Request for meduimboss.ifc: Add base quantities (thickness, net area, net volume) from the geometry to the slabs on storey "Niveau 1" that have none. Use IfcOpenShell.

First a look at what the model holds.

```python
import ifcopenshell
import ifcopenshell.util.element
import ifcopenshell.util.unit

model = ifcopenshell.open("meduimboss.ifc")
print(model.schema)
for unit_type in ("LENGTHUNIT", "AREAUNIT", "VOLUMEUNIT"):
    print(unit_type, ifcopenshell.util.unit.calculate_unit_scale(model, unit_type))
storey = next(s for s in model.by_type("IfcBuildingStorey") if s.Name == "Niveau 1")
slabs = [e for e in ifcopenshell.util.element.get_decomposition(storey) if e.is_a("IfcSlab")]
for e in sorted(slabs, key=lambda e: e.id()):
    print(e.id(), e.is_a(), e.Name, list(ifcopenshell.util.element.get_psets(e, qtos_only=True)), sep=" | ")
```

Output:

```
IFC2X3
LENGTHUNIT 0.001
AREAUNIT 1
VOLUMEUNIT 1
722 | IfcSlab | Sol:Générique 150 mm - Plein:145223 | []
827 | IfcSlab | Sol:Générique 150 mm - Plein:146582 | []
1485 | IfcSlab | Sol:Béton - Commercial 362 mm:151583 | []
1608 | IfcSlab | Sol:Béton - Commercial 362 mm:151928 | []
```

```python
import ifcopenshell
import ifcopenshell.api.pset
import ifcopenshell.geom
import ifcopenshell.util.element
import ifcopenshell.util.shape
import ifcopenshell.util.unit

model = ifcopenshell.open("meduimboss.ifc")
unit_scale = ifcopenshell.util.unit.calculate_unit_scale(model)
area_scale = ifcopenshell.util.unit.calculate_unit_scale(model, "AREAUNIT")
volume_scale = ifcopenshell.util.unit.calculate_unit_scale(model, "VOLUMEUNIT")
settings = ifcopenshell.geom.settings()

storey = next(s for s in model.by_type("IfcBuildingStorey") if s.Name == "Niveau 1")
slabs = [e for e in ifcopenshell.util.element.get_decomposition(storey) if e.is_a("IfcSlab")]

for e in sorted(slabs, key=lambda e: e.id()):
    if ifcopenshell.util.element.get_psets(e, qtos_only=True, should_inherit=False):
        continue
    # Geometry comes back in metres, in the element's own axes.
    shape = ifcopenshell.geom.create_shape(settings, e)
    values = {
        "Width": ifcopenshell.util.shape.get_z(shape.geometry) / unit_scale,
        "NetArea": ifcopenshell.util.shape.get_footprint_area(shape.geometry) / area_scale,
        "NetVolume": ifcopenshell.util.shape.get_volume(shape.geometry) / volume_scale,
    }
    qto = ifcopenshell.api.pset.add_qto(model, product=e, name="BaseQuantities")
    ifcopenshell.api.pset.edit_qto(model, qto=qto, properties=values)
    print(e.id(), {k: round(v, 3) for k, v in values.items()})

model.write("meduimboss_updated.ifc")
```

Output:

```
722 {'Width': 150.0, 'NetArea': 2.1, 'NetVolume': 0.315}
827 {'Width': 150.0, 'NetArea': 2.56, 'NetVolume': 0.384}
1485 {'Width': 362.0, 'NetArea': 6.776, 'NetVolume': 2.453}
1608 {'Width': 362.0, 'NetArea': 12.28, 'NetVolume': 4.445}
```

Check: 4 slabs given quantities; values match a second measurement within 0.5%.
